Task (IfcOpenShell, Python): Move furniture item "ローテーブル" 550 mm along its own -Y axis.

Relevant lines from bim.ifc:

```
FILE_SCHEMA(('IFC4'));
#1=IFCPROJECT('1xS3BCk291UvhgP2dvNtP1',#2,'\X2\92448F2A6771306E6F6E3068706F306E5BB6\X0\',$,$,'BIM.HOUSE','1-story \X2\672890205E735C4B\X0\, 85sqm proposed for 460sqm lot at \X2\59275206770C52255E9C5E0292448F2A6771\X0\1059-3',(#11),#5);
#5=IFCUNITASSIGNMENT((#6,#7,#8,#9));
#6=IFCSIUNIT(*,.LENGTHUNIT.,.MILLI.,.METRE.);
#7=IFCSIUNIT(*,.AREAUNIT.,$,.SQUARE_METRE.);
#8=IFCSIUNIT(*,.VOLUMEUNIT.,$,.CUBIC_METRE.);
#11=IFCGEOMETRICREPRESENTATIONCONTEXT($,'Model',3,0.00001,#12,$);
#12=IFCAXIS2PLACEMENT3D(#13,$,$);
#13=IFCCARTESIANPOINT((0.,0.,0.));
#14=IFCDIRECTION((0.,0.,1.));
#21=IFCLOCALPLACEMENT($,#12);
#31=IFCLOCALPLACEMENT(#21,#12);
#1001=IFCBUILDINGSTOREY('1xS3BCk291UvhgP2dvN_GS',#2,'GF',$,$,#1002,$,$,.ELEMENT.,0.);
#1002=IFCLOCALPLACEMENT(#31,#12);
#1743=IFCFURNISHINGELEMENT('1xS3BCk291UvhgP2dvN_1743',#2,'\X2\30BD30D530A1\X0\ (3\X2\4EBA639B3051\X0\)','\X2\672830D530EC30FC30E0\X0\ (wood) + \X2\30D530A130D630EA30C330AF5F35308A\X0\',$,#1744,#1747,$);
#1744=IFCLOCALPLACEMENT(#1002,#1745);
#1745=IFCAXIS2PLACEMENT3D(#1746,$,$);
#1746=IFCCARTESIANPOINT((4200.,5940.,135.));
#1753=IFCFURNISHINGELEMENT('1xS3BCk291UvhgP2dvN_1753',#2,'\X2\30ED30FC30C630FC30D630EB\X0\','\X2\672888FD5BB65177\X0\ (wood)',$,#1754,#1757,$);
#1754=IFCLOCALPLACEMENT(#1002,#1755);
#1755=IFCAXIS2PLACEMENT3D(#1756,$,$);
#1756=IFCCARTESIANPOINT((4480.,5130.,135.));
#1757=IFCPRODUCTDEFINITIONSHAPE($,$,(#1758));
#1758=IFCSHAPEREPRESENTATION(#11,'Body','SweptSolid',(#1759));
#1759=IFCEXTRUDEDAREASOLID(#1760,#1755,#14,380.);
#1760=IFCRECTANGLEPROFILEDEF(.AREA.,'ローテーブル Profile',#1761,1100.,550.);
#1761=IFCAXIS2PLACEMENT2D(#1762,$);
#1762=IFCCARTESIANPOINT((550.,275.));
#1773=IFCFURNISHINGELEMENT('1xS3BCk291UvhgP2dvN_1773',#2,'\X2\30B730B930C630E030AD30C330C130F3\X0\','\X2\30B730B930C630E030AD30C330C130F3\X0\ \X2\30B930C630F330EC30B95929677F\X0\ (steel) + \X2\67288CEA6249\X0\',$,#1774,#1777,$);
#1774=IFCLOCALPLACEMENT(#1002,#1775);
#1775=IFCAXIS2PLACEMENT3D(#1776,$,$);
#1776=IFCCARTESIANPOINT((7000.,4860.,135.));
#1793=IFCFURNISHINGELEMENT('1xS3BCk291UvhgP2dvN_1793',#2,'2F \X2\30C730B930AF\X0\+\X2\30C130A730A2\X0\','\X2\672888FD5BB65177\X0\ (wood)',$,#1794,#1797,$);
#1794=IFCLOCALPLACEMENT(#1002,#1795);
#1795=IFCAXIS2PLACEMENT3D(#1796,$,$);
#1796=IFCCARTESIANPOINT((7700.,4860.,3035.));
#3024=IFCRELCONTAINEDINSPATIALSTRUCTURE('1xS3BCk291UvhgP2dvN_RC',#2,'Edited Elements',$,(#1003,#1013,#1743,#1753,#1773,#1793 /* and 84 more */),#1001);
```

```python
import ifcopenshell
import ifcopenshell.api.geometry
import ifcopenshell.util.placement
import ifcopenshell.util.unit

model = ifcopenshell.open("bim.ifc")
unit_scale = ifcopenshell.util.unit.calculate_unit_scale(model)

item = model.by_id(1753)
matrix = ifcopenshell.util.placement.get_local_placement(item.ObjectPlacement)
matrix[:3, 3] -= matrix[:3, 1] * 0.55 / unit_scale
ifcopenshell.api.geometry.edit_object_placement(model, product=item, matrix=matrix, is_si=False)

print(ifcopenshell.util.placement.get_local_placement(item.ObjectPlacement).round(3) + 0.0)

model.write("bim_edited.ifc")
```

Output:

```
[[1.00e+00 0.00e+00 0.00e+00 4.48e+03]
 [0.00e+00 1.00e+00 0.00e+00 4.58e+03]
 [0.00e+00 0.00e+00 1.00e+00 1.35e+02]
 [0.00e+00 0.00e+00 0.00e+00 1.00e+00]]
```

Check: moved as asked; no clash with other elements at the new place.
